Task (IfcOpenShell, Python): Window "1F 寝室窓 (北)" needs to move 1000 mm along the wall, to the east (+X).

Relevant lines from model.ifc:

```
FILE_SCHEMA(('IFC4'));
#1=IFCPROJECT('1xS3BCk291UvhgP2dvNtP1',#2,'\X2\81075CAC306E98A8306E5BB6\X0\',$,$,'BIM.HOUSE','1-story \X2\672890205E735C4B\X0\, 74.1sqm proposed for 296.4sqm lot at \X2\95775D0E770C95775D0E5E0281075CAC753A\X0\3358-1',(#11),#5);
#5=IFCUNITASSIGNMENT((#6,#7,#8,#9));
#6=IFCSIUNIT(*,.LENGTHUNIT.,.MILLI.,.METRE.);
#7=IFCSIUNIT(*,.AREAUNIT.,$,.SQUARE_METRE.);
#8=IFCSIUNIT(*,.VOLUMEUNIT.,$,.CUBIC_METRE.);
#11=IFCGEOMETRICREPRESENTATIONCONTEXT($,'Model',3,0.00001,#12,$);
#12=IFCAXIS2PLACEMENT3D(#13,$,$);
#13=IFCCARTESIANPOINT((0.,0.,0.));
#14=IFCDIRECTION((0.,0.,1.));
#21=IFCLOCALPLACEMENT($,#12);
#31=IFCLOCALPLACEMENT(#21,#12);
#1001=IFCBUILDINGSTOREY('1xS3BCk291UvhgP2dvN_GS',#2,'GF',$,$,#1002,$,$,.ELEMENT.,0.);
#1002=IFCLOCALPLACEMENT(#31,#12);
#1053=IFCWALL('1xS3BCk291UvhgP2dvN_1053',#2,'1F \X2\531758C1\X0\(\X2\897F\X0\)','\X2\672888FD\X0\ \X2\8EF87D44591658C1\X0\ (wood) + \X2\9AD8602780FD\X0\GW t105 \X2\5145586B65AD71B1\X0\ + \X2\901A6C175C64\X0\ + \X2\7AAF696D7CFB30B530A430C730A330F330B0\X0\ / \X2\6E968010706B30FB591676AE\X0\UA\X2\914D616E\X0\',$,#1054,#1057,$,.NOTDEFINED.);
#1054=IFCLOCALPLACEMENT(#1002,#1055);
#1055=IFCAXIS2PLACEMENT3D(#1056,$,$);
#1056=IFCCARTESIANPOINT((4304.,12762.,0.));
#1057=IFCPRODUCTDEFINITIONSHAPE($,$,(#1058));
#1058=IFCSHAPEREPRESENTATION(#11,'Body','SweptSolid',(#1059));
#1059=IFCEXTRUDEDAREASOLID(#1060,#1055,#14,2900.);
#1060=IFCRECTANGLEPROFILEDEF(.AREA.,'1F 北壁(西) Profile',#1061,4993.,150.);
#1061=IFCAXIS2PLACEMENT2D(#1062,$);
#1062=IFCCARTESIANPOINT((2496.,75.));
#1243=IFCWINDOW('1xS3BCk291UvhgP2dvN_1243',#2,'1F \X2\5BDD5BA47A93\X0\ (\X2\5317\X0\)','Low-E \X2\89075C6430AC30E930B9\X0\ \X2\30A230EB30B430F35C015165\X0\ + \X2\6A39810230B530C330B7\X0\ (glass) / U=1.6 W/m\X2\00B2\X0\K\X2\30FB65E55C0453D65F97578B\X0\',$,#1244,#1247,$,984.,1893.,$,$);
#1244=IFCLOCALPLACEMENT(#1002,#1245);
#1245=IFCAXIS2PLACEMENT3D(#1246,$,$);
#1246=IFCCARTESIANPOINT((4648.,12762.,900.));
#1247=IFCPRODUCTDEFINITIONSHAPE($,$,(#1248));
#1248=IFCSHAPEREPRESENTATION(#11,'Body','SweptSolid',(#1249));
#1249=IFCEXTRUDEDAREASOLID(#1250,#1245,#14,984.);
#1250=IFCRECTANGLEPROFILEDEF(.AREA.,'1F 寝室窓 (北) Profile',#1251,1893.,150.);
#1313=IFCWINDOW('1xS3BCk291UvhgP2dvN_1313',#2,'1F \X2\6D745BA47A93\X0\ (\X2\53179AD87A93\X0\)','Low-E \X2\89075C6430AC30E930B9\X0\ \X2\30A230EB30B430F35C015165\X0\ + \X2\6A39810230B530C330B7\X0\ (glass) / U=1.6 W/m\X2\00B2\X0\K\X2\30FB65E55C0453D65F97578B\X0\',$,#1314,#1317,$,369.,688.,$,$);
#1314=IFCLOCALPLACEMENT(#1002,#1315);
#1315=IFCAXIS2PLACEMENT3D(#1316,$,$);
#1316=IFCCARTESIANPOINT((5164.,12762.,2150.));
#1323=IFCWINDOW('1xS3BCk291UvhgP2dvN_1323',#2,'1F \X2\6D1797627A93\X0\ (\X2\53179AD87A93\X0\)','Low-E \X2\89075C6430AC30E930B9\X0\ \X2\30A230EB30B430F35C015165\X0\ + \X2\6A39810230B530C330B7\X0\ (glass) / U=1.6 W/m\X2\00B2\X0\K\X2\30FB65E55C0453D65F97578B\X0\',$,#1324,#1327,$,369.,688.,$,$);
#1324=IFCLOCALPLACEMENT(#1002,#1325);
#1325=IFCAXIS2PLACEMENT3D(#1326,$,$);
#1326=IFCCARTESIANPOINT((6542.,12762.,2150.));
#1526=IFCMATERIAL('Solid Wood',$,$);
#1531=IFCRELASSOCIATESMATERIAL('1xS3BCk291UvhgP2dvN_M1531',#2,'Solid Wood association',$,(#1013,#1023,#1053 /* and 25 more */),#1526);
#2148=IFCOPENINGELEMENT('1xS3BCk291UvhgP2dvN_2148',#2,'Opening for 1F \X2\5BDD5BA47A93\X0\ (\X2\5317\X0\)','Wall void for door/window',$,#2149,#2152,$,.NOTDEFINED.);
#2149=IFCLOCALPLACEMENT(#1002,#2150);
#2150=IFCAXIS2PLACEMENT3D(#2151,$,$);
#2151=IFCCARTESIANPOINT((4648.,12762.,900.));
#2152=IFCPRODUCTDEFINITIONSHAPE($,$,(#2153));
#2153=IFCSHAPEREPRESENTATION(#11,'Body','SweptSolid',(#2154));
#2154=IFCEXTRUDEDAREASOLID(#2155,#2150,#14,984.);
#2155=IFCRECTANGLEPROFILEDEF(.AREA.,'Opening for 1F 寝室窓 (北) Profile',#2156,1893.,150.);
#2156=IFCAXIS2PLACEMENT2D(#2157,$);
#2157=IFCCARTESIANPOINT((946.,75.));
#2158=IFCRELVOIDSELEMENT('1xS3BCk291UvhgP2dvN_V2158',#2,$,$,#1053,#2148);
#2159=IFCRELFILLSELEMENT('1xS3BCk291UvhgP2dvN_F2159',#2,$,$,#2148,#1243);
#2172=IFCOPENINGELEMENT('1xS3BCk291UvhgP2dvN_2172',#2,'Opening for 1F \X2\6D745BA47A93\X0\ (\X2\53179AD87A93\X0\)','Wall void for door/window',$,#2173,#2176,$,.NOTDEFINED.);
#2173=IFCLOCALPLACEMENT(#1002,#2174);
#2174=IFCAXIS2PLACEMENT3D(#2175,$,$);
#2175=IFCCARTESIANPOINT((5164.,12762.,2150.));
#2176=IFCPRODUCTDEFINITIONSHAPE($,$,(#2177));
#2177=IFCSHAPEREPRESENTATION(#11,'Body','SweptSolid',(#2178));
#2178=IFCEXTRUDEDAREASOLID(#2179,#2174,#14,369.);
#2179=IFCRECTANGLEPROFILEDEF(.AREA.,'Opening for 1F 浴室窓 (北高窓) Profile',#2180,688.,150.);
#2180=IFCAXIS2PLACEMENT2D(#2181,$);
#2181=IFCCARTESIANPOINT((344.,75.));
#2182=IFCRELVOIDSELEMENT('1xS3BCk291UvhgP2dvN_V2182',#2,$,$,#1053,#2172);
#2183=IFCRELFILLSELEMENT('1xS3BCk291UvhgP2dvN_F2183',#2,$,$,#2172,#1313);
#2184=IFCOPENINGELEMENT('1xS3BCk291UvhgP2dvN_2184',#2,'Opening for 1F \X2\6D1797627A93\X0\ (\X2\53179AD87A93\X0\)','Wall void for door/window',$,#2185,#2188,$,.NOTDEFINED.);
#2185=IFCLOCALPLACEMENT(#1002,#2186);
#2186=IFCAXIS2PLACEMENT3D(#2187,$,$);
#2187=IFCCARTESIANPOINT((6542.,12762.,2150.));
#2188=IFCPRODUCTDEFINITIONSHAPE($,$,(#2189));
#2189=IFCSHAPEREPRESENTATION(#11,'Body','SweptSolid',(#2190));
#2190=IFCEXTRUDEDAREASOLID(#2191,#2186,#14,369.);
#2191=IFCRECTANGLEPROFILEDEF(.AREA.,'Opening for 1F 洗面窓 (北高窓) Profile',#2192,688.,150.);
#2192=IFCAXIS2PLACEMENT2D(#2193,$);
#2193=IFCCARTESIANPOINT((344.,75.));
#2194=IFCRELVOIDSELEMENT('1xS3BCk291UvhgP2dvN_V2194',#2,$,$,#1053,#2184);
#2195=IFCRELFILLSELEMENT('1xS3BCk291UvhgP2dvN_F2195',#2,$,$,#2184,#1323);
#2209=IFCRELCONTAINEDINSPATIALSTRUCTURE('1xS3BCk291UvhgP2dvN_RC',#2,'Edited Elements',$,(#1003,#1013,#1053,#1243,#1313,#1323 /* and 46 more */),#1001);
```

```python
import ifcopenshell
import ifcopenshell.api.geometry
import ifcopenshell.util.placement
import ifcopenshell.util.unit

model = ifcopenshell.open("model.ifc")
unit_scale = ifcopenshell.util.unit.calculate_unit_scale(model)

window = model.by_guid("1xS3BCk291UvhgP2dvN_1243")
opening = window.FillsVoids[0].RelatingOpeningElement
wall = opening.VoidsElements[0].RelatingBuildingElement

wall_matrix = ifcopenshell.util.placement.get_local_placement(wall.ObjectPlacement)
shift = wall_matrix[:3, 0] * 1 / unit_scale
before = ifcopenshell.util.placement.get_local_placement(window.ObjectPlacement)[:3, 3].copy()

# The window is not placed relative to its opening, so move both.
for product in (opening, window):
    matrix = ifcopenshell.util.placement.get_local_placement(product.ObjectPlacement)
    matrix[:3, 3] += shift
    ifcopenshell.api.geometry.edit_object_placement(model, product=product, matrix=matrix, is_si=False)

after = ifcopenshell.util.placement.get_local_placement(window.ObjectPlacement)[:3, 3]
print("window moved by", (after - before).round(3) + 0.0)

model.write("model_updated.ifc")
```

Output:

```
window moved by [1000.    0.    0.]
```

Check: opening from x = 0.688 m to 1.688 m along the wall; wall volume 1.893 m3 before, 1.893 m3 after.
